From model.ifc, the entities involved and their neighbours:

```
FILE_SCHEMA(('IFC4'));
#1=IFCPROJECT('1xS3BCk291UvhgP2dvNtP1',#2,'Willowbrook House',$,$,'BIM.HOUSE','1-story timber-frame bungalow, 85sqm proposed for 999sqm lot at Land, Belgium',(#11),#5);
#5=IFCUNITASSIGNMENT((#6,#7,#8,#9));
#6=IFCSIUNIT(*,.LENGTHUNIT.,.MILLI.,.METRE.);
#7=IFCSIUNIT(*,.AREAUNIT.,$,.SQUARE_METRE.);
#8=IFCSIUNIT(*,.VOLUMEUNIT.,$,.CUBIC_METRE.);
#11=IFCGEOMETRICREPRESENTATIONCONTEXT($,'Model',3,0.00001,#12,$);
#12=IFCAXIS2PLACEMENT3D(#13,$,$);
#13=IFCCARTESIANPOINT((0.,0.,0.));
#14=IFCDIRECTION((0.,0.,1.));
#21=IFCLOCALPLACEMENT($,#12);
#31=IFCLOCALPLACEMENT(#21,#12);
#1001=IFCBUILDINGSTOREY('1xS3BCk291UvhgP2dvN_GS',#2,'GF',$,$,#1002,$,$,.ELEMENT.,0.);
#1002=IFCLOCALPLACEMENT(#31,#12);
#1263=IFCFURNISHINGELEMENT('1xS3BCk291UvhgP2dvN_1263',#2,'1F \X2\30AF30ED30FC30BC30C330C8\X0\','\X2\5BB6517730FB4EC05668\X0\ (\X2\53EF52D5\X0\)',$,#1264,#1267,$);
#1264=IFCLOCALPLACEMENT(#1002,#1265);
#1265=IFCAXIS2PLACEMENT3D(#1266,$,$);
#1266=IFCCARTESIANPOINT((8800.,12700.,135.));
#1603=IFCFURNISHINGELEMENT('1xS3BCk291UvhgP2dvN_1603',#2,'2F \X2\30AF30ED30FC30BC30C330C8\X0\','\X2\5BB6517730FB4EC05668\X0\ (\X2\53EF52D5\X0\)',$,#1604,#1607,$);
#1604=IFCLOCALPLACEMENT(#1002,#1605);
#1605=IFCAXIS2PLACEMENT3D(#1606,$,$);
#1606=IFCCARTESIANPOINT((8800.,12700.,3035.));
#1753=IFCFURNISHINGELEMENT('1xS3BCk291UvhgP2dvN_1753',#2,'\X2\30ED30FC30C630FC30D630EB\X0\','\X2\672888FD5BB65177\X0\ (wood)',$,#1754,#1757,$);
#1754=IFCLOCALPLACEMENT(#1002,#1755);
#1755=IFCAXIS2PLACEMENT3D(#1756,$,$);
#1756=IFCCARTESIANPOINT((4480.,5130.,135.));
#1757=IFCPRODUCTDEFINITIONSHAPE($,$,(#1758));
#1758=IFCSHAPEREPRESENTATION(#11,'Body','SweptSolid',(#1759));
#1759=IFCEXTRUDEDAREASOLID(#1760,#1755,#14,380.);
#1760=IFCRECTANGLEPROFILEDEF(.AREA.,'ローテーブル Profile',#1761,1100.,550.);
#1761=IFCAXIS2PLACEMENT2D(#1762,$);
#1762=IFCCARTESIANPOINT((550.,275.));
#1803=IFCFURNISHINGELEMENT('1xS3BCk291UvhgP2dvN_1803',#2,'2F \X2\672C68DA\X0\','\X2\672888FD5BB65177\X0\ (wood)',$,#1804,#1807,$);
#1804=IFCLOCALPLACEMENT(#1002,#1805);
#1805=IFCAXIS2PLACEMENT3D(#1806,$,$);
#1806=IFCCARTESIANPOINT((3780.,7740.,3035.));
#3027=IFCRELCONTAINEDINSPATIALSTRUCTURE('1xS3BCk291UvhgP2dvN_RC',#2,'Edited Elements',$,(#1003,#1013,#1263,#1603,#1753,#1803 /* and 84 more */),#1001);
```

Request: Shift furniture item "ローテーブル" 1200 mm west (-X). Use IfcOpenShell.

```python
import ifcopenshell
import ifcopenshell.api.geometry
import ifcopenshell.util.placement
import ifcopenshell.util.unit

model = ifcopenshell.open("model.ifc")
unit_scale = ifcopenshell.util.unit.calculate_unit_scale(model)

item = model.by_guid("1xS3BCk291UvhgP2dvN_1753")
matrix = ifcopenshell.util.placement.get_local_placement(item.ObjectPlacement)
matrix[0, 3] -= 1.2 / unit_scale
ifcopenshell.api.geometry.edit_object_placement(model, product=item, matrix=matrix, is_si=False)

print(ifcopenshell.util.placement.get_local_placement(item.ObjectPlacement).round(3) + 0.0)

model.write("model_edited.ifc")
```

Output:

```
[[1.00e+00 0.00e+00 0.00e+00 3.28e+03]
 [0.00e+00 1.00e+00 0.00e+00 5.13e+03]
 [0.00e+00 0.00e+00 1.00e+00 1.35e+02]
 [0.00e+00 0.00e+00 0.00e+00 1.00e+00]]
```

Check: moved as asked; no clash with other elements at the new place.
